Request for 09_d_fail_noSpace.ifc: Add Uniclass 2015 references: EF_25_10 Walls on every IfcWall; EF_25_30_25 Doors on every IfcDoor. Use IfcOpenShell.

First a look at what the model holds.

```python
import ifcopenshell

model = ifcopenshell.open("09_d_fail_noSpace.ifc")
print(model.schema)
print("classifications:", [c.Name for c in model.by_type("IfcClassification")])
for ifc_class in ("IfcDoor", "IfcRoof", "IfcStair", "IfcWall", "IfcWindow"):
    print(ifc_class, len(model.by_type(ifc_class)))
```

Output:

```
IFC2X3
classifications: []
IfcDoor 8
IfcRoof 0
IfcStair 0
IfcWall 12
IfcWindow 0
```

```python
import ifcopenshell
import ifcopenshell.api.classification

model = ifcopenshell.open("09_d_fail_noSpace.ifc")

# IFC2X3 requires Source and Edition and has no link from the project to the system.
system = model.create_entity("IfcClassification", Source="NBS", Edition="2015", Name="Uniclass 2015")

codes = {
    "IfcWall": ("EF_25_10", "Walls"),
    "IfcDoor": ("EF_25_30_25", "Doors"),
}
for ifc_class, (code, name) in codes.items():
    products = model.by_type(ifc_class)
    ifcopenshell.api.classification.add_reference(
        model, products=products, classification=system, identification=code, name=name
    )
    print(code, len(products))

model.write("09_d_fail_noSpace_edited.ifc")
```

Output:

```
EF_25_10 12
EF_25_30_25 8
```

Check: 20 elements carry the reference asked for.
